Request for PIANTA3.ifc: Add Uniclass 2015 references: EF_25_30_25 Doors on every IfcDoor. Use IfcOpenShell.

First a look at what the model holds.

```python
import ifcopenshell

model = ifcopenshell.open("PIANTA3.ifc")
print(model.schema)
print("classifications:", [c.Name for c in model.by_type("IfcClassification")])
for ifc_class in ("IfcDoor", "IfcRoof", "IfcStair", "IfcWall", "IfcWindow"):
    print(ifc_class, len(model.by_type(ifc_class)))
```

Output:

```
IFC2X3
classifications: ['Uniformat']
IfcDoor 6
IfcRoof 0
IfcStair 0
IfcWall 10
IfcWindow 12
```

```python
import ifcopenshell
import ifcopenshell.api.classification

model = ifcopenshell.open("PIANTA3.ifc")

# IFC2X3 requires Source and Edition and has no link from the project to the system.
system = model.create_entity("IfcClassification", Source="NBS", Edition="2015", Name="Uniclass 2015")

codes = {
    "IfcDoor": ("EF_25_30_25", "Doors"),
}
for ifc_class, (code, name) in codes.items():
    products = model.by_type(ifc_class)
    ifcopenshell.api.classification.add_reference(
        model, products=products, classification=system, identification=code, name=name
    )
    print(code, len(products))

model.write("PIANTA3-out.ifc")
```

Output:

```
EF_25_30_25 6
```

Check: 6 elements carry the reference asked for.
